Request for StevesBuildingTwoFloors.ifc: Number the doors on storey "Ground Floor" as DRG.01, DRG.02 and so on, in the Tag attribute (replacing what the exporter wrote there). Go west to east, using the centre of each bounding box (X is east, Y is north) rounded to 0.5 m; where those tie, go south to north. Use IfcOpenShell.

First a look at what the model holds.

```python
import ifcopenshell
import ifcopenshell.util.element
import ifcopenshell.util.placement

model = ifcopenshell.open("StevesBuildingTwoFloors.ifc")
print(model.schema)
storey = next(s for s in model.by_type("IfcBuildingStorey") if s.Name == "Ground Floor")
doors = [e for e in ifcopenshell.util.element.get_decomposition(storey) if e.is_a("IfcDoor")]
for e in sorted(doors, key=lambda e: e.id()):
    origin = ifcopenshell.util.placement.get_local_placement(e.ObjectPlacement)[:3, 3]
    print(e.id(), e.Tag, e.Name, origin.round(2) + 0.0, sep=" | ")
```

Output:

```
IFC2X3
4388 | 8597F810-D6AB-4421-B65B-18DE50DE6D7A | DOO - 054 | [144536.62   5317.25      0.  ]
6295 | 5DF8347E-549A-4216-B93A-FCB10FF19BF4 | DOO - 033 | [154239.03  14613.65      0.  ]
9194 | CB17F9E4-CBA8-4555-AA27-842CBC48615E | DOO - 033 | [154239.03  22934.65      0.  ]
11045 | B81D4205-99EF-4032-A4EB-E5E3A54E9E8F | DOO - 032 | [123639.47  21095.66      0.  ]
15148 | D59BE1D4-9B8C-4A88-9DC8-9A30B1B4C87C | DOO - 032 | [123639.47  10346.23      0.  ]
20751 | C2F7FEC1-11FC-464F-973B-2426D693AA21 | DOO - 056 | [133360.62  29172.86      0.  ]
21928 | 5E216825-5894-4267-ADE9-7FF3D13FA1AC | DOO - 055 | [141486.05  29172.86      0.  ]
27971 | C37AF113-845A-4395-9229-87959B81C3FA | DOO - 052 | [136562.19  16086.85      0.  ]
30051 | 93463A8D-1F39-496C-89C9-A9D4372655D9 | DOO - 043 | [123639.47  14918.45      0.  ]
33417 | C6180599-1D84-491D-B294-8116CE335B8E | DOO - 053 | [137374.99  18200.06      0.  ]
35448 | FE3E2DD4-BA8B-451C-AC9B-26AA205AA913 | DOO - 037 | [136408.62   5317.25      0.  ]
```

```python
import ifcopenshell
import ifcopenshell.geom
import ifcopenshell.util.element
import ifcopenshell.util.shape

model = ifcopenshell.open("StevesBuildingTwoFloors.ifc")
settings = ifcopenshell.geom.settings()
settings.set("use-world-coords", True)


def centre(element):
    shape = ifcopenshell.geom.create_shape(settings, element)
    return ifcopenshell.util.shape.get_bbox_centroid(shape.geometry)


storey = next(s for s in model.by_type("IfcBuildingStorey") if s.Name == "Ground Floor")
doors = [e for e in ifcopenshell.util.element.get_decomposition(storey) if e.is_a("IfcDoor")]

# Insertion points can sit at a corner or the storey origin, so sort by the geometry (in metres).
centres = {e: centre(e) for e in doors}
doors.sort(key=lambda e: (round(centres[e][0] / 0.5), centres[e][1]))

for i, e in enumerate(doors, start=1):
    number = f"DRG.{i:02d}"
    e.Tag = number
    print(e.id(), number)

model.write("StevesBuildingTwoFloors_updated.ifc")
```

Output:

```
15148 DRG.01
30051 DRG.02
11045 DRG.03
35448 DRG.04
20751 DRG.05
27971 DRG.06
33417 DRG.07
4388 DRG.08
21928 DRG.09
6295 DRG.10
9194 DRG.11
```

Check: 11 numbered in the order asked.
